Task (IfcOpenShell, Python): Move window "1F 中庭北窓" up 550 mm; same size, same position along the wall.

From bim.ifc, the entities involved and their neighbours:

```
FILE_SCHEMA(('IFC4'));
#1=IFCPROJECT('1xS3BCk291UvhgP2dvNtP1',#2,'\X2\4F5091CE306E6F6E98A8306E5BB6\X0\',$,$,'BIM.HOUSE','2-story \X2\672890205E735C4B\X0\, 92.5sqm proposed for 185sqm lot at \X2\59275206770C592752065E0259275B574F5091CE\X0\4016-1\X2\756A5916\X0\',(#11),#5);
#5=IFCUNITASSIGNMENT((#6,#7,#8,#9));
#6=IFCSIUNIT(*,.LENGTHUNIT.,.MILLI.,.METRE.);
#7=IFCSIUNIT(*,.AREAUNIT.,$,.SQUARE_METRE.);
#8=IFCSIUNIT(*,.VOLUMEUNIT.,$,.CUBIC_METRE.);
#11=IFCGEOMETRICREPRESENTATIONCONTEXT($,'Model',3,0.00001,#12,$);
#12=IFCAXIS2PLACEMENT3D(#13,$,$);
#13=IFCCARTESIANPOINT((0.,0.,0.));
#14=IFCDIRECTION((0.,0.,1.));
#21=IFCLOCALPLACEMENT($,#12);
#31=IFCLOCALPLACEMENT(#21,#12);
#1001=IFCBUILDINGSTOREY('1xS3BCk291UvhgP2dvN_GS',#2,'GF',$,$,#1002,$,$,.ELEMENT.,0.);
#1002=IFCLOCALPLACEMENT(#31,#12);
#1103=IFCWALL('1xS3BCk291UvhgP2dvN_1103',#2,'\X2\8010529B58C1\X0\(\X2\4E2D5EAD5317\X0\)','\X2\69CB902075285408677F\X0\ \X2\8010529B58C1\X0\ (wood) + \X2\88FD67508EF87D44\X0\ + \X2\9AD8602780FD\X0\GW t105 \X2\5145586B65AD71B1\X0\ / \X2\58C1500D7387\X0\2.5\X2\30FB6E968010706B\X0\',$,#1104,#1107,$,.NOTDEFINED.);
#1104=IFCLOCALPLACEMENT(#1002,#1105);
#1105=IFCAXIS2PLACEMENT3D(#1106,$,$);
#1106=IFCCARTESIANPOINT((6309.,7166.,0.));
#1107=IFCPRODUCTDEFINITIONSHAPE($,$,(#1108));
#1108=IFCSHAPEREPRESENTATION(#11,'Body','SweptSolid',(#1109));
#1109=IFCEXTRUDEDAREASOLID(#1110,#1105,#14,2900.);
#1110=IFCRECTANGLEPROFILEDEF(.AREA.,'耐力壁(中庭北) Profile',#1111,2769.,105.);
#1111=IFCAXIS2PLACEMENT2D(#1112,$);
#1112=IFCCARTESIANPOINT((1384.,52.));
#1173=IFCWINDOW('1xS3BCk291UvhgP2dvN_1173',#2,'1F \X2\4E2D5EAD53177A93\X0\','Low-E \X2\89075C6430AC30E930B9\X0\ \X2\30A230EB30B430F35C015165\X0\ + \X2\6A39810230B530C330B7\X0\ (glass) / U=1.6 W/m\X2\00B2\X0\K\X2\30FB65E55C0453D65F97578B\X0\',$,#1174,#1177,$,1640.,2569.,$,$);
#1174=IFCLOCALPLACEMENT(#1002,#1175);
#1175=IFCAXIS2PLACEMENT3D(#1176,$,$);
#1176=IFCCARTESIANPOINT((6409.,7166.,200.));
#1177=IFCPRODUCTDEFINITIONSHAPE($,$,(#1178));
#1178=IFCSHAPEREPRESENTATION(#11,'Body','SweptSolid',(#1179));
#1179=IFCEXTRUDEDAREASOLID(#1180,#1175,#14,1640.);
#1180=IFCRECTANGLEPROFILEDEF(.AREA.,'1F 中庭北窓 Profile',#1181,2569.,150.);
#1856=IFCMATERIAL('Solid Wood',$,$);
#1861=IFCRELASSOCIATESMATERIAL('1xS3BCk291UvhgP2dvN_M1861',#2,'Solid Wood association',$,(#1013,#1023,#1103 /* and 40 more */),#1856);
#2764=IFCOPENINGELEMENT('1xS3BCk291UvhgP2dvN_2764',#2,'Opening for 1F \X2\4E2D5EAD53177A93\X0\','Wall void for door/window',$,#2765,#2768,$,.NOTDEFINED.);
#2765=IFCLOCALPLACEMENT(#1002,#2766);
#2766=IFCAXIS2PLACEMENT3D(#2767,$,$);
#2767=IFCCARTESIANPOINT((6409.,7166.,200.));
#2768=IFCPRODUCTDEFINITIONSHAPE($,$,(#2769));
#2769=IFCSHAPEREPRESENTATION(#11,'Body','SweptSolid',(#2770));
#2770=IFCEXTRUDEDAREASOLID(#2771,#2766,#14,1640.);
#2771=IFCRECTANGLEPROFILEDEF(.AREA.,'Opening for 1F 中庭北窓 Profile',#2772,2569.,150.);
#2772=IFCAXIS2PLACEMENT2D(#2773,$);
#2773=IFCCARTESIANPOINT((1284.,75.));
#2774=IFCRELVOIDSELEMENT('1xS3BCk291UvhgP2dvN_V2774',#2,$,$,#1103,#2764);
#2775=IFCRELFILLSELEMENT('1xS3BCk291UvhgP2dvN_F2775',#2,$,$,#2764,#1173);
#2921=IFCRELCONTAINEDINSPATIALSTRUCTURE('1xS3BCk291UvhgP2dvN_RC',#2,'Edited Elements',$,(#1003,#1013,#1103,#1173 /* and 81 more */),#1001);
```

```python
import numpy as np
import ifcopenshell
import ifcopenshell.api.geometry
import ifcopenshell.util.placement
import ifcopenshell.util.unit

model = ifcopenshell.open("bim.ifc")
unit_scale = ifcopenshell.util.unit.calculate_unit_scale(model)

window = model.by_guid("1xS3BCk291UvhgP2dvN_1173")
opening = window.FillsVoids[0].RelatingOpeningElement
dz = 550.0

shift = np.array([0.0, 0.0, dz])
# The window is not placed relative to its opening, so move both.
for product in (opening, window):
    matrix = ifcopenshell.util.placement.get_local_placement(product.ObjectPlacement)
    matrix[:3, 3] += shift
    ifcopenshell.api.geometry.edit_object_placement(model, product=product, matrix=matrix, is_si=False)

print(f"moved by {dz * unit_scale:+.3f} m")

model.write("bim_updated.ifc")
```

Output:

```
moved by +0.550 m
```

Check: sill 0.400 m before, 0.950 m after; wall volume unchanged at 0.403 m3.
